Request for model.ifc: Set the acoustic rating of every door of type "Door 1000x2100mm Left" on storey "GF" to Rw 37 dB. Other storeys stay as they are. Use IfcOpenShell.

First a look at what the model holds.

```python
import ifcopenshell
import ifcopenshell.util.element

model = ifcopenshell.open("model.ifc")
print(model.schema)
storey = next(s for s in model.by_type("IfcBuildingStorey") if s.Name == "GF")
doors = [e for e in ifcopenshell.util.element.get_decomposition(storey) if e.is_a("IfcDoor")]
seen = {}
for e in doors:
    element_type = ifcopenshell.util.element.get_type(e)
    key = (element_type.Name if element_type != e and element_type else None, ifcopenshell.util.element.get_pset(e, "Pset_DoorCommon", "AcousticRating"))
    seen[key] = seen.get(key, 0) + 1
for (name, value), count in sorted(seen.items(), key=str):
    print(count, "x", name, "|", value)
```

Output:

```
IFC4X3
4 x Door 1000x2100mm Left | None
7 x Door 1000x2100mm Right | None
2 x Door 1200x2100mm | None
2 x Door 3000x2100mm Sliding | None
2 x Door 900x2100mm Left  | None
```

```python
import ifcopenshell
import ifcopenshell.api.pset
import ifcopenshell.util.element

model = ifcopenshell.open("model.ifc")

storey = next(s for s in model.by_type("IfcBuildingStorey") if s.Name == "GF")
doors = [e for e in ifcopenshell.util.element.get_decomposition(storey) if e.is_a("IfcDoor")]

count = 0
for e in doors:
    element_type = ifcopenshell.util.element.get_type(e)
    if element_type in (None, e) or element_type.Name != "Door 1000x2100mm Left":
        continue
    # add_pset returns the element's existing set when there is one.
    pset = ifcopenshell.api.pset.add_pset(model, product=e, name="Pset_DoorCommon")
    ifcopenshell.api.pset.edit_pset(model, pset=pset, properties={"AcousticRating": "Rw 37 dB"})
    count += 1

print(count, "doors updated")

model.write("model-out.ifc")
```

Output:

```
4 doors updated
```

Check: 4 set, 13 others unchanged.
